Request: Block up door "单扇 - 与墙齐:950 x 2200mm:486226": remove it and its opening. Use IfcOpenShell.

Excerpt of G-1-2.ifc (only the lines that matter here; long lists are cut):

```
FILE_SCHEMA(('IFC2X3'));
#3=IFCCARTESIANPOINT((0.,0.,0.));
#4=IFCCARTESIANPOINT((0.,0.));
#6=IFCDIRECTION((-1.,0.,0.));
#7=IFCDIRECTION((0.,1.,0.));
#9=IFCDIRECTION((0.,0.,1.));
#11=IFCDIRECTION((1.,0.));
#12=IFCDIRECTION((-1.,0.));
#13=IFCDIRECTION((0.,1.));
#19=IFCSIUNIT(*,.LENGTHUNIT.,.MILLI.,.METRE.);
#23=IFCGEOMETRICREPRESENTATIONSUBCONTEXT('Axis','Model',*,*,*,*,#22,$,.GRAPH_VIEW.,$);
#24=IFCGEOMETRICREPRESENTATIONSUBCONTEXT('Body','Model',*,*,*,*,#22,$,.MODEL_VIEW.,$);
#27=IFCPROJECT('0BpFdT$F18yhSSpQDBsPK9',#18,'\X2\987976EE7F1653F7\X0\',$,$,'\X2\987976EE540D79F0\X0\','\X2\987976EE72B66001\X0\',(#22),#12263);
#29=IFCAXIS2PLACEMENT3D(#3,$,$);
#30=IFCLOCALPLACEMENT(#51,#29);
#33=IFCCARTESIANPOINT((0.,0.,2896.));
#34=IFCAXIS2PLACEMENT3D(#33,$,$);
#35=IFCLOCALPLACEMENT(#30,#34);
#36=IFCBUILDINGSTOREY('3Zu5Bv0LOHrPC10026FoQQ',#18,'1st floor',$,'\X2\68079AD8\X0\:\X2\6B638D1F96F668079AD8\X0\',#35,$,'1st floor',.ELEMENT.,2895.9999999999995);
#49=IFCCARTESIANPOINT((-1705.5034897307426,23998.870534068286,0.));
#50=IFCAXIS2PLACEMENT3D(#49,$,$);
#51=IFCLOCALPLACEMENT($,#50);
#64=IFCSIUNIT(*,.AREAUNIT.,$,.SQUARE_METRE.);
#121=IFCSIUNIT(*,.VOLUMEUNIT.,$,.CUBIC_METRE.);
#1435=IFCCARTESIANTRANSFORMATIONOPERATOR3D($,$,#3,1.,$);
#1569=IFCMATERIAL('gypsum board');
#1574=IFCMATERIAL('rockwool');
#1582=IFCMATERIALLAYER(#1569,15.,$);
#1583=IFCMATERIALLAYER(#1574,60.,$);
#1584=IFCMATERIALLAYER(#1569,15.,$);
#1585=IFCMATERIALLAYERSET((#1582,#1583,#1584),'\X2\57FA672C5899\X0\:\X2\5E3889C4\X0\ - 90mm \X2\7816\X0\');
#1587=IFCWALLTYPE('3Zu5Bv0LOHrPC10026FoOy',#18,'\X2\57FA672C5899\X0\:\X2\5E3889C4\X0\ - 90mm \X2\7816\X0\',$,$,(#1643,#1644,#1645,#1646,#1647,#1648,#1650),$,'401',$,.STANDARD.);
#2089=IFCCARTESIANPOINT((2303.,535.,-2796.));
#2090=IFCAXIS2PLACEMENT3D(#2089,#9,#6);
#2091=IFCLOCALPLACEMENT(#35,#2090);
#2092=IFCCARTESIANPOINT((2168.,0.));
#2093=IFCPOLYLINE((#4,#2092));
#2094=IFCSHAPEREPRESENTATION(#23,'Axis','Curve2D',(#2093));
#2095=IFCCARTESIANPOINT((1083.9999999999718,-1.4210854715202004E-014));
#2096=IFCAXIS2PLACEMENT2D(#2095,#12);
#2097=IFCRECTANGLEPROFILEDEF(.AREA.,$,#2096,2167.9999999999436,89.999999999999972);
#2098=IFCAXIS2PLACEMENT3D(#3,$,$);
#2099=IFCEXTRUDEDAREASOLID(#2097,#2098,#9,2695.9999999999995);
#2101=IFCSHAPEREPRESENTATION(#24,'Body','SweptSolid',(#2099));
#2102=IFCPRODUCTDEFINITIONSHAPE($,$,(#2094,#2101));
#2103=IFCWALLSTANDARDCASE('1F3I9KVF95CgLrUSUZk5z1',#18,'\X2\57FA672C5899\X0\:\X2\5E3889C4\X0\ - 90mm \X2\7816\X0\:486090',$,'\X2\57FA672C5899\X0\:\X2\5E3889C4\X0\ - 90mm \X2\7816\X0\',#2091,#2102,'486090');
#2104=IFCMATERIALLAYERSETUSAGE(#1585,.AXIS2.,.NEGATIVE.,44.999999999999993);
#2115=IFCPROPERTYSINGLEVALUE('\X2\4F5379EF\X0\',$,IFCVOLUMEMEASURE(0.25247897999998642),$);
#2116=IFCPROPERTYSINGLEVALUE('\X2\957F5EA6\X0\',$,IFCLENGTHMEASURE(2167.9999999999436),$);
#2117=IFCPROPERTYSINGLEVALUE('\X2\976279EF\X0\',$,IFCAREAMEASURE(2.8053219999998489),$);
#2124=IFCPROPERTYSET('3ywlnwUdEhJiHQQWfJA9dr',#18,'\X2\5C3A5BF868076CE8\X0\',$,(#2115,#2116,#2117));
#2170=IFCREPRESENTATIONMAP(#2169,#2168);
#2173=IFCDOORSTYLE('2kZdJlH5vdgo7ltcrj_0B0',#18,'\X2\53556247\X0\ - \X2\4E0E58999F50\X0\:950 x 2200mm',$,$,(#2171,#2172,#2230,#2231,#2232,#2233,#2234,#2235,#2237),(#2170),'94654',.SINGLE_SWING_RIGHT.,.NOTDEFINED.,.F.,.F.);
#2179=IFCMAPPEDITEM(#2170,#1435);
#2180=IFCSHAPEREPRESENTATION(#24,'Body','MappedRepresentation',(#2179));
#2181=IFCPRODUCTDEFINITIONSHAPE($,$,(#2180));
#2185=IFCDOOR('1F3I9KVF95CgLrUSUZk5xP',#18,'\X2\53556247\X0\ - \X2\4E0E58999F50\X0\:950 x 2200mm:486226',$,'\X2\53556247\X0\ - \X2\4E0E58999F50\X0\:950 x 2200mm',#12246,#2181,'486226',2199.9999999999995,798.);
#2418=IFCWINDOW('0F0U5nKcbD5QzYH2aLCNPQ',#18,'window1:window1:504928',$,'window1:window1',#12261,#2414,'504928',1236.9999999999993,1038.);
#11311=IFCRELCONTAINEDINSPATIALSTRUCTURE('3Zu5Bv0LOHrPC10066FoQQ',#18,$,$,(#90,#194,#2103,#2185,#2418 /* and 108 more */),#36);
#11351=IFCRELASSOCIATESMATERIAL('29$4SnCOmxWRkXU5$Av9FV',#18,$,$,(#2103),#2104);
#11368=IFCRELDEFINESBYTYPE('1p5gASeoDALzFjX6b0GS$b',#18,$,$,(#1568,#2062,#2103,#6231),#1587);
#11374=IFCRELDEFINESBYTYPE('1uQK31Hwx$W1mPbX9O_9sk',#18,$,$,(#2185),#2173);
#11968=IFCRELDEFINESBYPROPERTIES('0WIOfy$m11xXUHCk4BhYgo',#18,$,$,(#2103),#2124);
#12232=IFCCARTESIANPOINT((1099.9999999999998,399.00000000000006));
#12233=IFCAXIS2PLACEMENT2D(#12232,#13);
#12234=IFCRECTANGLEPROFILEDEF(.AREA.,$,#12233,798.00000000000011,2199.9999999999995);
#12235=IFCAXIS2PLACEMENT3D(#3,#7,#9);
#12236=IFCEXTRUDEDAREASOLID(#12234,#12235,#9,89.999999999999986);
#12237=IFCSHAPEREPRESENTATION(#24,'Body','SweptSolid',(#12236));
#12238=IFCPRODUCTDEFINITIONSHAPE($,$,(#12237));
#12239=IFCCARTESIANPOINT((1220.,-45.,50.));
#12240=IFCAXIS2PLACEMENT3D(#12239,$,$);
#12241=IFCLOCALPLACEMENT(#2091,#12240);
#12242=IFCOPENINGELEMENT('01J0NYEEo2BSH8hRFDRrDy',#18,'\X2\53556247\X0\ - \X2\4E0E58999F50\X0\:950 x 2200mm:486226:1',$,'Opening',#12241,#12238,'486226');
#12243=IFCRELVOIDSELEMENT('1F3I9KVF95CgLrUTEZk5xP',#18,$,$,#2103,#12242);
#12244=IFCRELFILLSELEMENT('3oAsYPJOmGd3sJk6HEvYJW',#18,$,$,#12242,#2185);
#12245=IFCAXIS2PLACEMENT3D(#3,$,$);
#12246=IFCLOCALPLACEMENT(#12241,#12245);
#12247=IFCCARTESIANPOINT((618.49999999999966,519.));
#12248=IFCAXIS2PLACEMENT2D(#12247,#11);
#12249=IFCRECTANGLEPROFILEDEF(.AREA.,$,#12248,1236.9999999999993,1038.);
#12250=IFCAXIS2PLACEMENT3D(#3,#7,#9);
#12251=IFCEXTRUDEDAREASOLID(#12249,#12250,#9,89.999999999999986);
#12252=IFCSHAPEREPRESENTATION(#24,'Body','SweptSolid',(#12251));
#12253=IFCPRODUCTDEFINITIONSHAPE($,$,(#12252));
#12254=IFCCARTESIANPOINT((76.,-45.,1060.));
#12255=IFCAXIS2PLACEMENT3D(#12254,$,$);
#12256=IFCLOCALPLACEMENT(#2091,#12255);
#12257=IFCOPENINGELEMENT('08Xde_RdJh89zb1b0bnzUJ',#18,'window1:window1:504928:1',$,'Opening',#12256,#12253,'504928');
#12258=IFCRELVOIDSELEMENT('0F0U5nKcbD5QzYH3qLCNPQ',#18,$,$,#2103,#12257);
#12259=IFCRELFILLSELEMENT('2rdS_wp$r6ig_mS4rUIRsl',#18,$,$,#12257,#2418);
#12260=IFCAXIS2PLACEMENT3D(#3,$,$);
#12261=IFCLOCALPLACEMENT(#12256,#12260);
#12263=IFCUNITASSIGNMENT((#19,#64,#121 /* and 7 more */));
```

```python
import ifcopenshell
import ifcopenshell.api.feature
import ifcopenshell.api.pset
import ifcopenshell.api.root
import ifcopenshell.geom
import ifcopenshell.util.element
import ifcopenshell.util.shape
import ifcopenshell.util.unit

model = ifcopenshell.open("G-1-2.ifc")
area_scale = ifcopenshell.util.unit.calculate_unit_scale(model, "AREAUNIT")
volume_scale = ifcopenshell.util.unit.calculate_unit_scale(model, "VOLUMEUNIT")
settings = ifcopenshell.geom.settings()


def volume(element):
    """Net volume in cubic metres, openings subtracted."""
    shape = ifcopenshell.geom.create_shape(settings, element)
    return ifcopenshell.util.shape.get_volume(shape.geometry)


door = model.by_guid("1F3I9KVF95CgLrUSUZk5xP")
opening = door.FillsVoids[0].RelatingOpeningElement
wall = opening.VoidsElements[0].RelatingBuildingElement
before = volume(wall)

ifcopenshell.api.root.remove_product(model, product=door)
ifcopenshell.api.feature.remove_feature(model, feature=opening)

after = volume(wall)
thickness = 0.09  # wall thickness in metres

# Update the wall's stored quantities.
pset = model.by_id(ifcopenshell.util.element.get_pset(wall, "尺寸标注", should_inherit=False)["id"])
ifcopenshell.api.pset.edit_pset(model, pset=pset, properties={
    "体积": model.create_entity("IfcVolumeMeasure", after / volume_scale),
    "面积": model.create_entity("IfcAreaMeasure", after / thickness / area_scale),
})

print(f"wall volume {before:.3f} -> {after:.3f} m3")

model.write("G-1-2_rev.ifc")
```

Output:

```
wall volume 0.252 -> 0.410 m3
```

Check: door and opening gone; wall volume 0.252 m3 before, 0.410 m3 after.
